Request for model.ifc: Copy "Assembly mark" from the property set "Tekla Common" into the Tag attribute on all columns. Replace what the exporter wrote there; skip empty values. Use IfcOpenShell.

First a look at what the model holds.

```python
import ifcopenshell
import ifcopenshell.util.element

model = ifcopenshell.open("model.ifc")
print(model.schema)
columns = model.by_type("IfcColumn")
print(len(columns), "columns")
for e in columns[:8]:
    source = ifcopenshell.util.element.get_pset(e, "Tekla Common", "Assembly mark")
    target = e.Tag
    print(e.id(), repr(source), repr(target), sep=" | ")
```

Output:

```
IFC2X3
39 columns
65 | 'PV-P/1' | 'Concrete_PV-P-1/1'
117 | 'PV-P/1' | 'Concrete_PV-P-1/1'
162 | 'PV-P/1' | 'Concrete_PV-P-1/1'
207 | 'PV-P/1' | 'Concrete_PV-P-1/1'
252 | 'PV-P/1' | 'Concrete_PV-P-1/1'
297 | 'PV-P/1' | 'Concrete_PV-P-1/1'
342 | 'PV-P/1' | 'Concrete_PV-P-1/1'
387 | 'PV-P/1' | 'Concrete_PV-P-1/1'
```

```python
import ifcopenshell
import ifcopenshell.util.element

model = ifcopenshell.open("model.ifc")

count = 0
for e in model.by_type("IfcColumn"):
    value = ifcopenshell.util.element.get_pset(e, "Tekla Common", "Assembly mark")
    current = e.Tag
    if not value or not value.strip() or current == value:
        continue
    e.Tag = value
    count += 1

print(count, "columns updated")

model.write("model-out.ifc")
```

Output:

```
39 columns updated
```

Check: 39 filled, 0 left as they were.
